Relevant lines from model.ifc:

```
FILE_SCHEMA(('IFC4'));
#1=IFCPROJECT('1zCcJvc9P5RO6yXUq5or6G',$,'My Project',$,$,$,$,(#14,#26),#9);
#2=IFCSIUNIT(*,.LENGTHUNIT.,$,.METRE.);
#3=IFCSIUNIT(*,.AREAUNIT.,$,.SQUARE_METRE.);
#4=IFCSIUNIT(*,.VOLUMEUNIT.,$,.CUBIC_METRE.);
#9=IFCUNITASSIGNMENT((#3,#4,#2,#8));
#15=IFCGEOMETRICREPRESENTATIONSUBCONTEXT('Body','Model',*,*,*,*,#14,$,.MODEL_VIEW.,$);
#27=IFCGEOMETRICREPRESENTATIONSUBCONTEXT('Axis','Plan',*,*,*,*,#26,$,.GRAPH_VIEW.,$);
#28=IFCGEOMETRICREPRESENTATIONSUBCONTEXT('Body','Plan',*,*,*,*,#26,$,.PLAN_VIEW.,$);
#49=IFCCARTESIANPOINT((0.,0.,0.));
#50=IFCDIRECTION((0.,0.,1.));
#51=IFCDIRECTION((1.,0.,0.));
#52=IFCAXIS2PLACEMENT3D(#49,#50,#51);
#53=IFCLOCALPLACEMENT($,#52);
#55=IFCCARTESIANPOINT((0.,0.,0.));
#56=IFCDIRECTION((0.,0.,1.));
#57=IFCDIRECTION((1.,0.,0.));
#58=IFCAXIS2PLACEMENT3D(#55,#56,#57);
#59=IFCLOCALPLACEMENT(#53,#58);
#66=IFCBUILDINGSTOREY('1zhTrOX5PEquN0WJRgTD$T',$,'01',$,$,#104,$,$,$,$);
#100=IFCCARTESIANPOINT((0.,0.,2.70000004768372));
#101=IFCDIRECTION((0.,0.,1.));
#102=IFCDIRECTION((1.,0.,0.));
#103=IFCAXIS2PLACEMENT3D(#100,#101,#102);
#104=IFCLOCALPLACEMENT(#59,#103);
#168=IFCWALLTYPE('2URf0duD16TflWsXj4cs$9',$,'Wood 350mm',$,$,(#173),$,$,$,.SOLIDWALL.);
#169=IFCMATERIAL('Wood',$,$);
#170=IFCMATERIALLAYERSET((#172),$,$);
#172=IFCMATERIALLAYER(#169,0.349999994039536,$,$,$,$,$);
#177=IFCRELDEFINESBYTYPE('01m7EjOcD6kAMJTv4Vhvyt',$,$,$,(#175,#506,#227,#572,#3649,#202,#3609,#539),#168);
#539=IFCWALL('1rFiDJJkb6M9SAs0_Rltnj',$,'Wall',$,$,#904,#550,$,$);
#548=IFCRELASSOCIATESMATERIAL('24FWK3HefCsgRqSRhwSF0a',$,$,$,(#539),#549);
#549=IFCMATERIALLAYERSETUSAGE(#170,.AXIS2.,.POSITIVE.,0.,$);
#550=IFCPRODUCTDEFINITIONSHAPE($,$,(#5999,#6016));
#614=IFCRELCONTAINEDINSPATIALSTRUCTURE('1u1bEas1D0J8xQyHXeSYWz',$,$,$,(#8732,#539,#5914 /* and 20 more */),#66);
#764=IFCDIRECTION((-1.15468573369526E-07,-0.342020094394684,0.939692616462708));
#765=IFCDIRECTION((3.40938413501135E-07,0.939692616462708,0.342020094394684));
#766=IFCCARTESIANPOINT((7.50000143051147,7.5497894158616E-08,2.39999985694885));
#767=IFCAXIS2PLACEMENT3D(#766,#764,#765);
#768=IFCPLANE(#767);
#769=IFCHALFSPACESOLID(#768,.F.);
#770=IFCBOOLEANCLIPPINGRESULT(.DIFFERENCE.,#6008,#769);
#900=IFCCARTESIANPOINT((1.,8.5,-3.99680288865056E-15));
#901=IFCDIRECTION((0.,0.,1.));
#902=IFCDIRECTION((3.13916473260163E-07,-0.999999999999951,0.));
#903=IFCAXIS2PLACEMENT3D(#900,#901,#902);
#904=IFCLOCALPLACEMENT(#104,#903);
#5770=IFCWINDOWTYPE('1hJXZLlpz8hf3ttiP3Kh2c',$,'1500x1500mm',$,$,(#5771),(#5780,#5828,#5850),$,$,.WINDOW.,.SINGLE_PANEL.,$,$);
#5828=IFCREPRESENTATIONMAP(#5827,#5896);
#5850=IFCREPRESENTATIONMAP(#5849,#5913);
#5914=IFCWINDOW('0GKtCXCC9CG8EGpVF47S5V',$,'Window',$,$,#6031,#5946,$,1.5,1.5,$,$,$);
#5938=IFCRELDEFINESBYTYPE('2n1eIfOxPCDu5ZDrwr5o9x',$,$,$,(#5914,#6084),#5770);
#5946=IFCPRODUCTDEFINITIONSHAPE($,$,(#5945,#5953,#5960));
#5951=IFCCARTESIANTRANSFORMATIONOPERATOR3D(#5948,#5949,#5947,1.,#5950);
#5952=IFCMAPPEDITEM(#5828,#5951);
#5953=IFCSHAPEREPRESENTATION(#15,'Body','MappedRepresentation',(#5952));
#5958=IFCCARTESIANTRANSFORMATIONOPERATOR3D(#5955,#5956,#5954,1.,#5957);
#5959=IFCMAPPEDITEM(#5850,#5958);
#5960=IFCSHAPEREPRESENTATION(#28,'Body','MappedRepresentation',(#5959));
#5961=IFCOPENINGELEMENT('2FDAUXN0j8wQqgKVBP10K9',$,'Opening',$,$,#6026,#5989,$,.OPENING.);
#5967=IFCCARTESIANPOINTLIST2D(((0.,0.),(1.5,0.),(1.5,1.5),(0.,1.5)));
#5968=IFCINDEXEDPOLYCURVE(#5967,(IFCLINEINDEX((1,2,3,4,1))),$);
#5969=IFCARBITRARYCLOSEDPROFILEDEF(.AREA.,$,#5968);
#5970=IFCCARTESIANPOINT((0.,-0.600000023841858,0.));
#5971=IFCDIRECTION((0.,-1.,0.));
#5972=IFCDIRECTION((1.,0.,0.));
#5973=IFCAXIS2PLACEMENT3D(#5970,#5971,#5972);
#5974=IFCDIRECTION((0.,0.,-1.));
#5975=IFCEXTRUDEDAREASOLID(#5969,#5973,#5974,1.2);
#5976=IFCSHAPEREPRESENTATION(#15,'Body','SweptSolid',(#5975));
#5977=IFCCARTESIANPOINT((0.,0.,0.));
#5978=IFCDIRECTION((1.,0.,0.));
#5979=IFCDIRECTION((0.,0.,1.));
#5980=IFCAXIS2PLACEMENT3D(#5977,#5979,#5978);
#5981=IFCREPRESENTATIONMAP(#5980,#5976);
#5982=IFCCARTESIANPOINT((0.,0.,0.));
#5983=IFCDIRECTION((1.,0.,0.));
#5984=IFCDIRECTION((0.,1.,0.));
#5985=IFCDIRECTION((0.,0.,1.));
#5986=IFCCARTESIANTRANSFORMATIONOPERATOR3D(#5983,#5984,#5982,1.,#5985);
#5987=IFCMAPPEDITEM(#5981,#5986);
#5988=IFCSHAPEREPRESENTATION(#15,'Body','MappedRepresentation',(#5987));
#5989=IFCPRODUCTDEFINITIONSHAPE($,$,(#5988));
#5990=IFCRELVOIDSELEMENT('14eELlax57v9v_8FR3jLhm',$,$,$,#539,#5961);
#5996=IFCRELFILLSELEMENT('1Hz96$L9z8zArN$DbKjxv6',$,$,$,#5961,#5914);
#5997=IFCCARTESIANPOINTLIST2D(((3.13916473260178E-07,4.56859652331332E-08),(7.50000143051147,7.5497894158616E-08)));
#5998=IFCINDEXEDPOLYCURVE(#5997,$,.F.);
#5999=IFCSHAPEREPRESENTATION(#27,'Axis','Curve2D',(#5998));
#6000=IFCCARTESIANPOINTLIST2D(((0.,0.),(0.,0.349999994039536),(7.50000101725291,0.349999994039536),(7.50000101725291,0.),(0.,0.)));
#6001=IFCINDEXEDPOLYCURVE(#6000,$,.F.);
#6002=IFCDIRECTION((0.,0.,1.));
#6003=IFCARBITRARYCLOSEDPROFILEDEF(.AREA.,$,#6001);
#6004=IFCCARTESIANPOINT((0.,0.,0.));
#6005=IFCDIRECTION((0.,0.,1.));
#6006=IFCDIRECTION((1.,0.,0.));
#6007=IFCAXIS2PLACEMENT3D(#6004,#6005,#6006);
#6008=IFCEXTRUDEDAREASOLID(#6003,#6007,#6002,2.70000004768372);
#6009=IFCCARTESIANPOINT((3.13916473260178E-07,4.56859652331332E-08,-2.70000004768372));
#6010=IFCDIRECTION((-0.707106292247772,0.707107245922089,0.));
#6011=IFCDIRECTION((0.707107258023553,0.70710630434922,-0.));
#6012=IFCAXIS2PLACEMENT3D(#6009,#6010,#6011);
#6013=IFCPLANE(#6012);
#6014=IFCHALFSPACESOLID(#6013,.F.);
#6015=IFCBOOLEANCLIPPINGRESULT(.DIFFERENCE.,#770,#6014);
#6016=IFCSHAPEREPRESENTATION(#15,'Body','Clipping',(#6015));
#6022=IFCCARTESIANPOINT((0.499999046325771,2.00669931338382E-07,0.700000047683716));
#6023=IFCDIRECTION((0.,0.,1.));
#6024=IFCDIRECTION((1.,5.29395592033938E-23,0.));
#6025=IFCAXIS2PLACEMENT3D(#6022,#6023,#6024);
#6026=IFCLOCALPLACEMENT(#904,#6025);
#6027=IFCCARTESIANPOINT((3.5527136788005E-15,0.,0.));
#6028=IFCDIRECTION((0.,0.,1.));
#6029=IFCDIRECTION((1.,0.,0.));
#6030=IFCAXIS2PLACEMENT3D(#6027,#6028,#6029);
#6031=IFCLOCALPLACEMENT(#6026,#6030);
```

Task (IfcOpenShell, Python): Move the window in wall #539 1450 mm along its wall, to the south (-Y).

```python
import ifcopenshell
import ifcopenshell.api.geometry
import ifcopenshell.util.placement

model = ifcopenshell.open("model.ifc")

window = model.by_id(5914)
opening = window.FillsVoids[0].RelatingOpeningElement
wall = opening.VoidsElements[0].RelatingBuildingElement

wall_matrix = ifcopenshell.util.placement.get_local_placement(wall.ObjectPlacement)
shift = wall_matrix[:3, 0] * 1.45
before = ifcopenshell.util.placement.get_local_placement(window.ObjectPlacement)[:3, 3].copy()

# The window is placed relative to its opening, so it follows when the opening moves.
matrix = ifcopenshell.util.placement.get_local_placement(opening.ObjectPlacement)
matrix[:3, 3] += shift
ifcopenshell.api.geometry.edit_object_placement(
    model, product=opening, matrix=matrix, is_si=False, should_transform_children=True
)

after = ifcopenshell.util.placement.get_local_placement(window.ObjectPlacement)[:3, 3]
print("window moved by", (after - before).round(3) + 0.0)

model.write("model-out.ifc")
```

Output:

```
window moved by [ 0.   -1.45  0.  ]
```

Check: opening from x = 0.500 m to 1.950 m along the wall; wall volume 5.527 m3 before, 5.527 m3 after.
